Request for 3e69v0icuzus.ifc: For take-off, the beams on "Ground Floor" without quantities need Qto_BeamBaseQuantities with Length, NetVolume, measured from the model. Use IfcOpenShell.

First a look at what the model holds.

```python
import ifcopenshell
import ifcopenshell.util.element
import ifcopenshell.util.unit

model = ifcopenshell.open("3e69v0icuzus.ifc")
print(model.schema)
for unit_type in ("LENGTHUNIT", "AREAUNIT", "VOLUMEUNIT"):
    print(unit_type, ifcopenshell.util.unit.calculate_unit_scale(model, unit_type))
storey = next(s for s in model.by_type("IfcBuildingStorey") if s.Name == "Ground Floor")
beams = [e for e in ifcopenshell.util.element.get_decomposition(storey) if e.is_a("IfcBeam")]
for e in sorted(beams, key=lambda e: e.id()):
    print(e.id(), e.is_a(), e.Name, list(ifcopenshell.util.element.get_psets(e, qtos_only=True)), sep=" | ")
```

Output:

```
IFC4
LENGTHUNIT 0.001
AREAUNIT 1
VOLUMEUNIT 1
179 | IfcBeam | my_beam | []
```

```python
import ifcopenshell
import ifcopenshell.api.pset
import ifcopenshell.geom
import ifcopenshell.util.element
import ifcopenshell.util.shape
import ifcopenshell.util.unit

model = ifcopenshell.open("3e69v0icuzus.ifc")
unit_scale = ifcopenshell.util.unit.calculate_unit_scale(model)
volume_scale = ifcopenshell.util.unit.calculate_unit_scale(model, "VOLUMEUNIT")
settings = ifcopenshell.geom.settings()

storey = next(s for s in model.by_type("IfcBuildingStorey") if s.Name == "Ground Floor")
beams = [e for e in ifcopenshell.util.element.get_decomposition(storey) if e.is_a("IfcBeam")]

for e in sorted(beams, key=lambda e: e.id()):
    if ifcopenshell.util.element.get_psets(e, qtos_only=True, should_inherit=False):
        continue
    # Geometry comes back in metres, in the element's own axes.
    shape = ifcopenshell.geom.create_shape(settings, e)
    values = {
        "Length": ifcopenshell.util.shape.get_max_xyz(shape.geometry) / unit_scale,
        "NetVolume": ifcopenshell.util.shape.get_volume(shape.geometry) / volume_scale,
    }
    qto = ifcopenshell.api.pset.add_qto(model, product=e, name="Qto_BeamBaseQuantities")
    ifcopenshell.api.pset.edit_qto(model, qto=qto, properties=values)
    print(e.id(), {k: round(v, 3) for k, v in values.items()})

model.write("3e69v0icuzus_updated.ifc")
```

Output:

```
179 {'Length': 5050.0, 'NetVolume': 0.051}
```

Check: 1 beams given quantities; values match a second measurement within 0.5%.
